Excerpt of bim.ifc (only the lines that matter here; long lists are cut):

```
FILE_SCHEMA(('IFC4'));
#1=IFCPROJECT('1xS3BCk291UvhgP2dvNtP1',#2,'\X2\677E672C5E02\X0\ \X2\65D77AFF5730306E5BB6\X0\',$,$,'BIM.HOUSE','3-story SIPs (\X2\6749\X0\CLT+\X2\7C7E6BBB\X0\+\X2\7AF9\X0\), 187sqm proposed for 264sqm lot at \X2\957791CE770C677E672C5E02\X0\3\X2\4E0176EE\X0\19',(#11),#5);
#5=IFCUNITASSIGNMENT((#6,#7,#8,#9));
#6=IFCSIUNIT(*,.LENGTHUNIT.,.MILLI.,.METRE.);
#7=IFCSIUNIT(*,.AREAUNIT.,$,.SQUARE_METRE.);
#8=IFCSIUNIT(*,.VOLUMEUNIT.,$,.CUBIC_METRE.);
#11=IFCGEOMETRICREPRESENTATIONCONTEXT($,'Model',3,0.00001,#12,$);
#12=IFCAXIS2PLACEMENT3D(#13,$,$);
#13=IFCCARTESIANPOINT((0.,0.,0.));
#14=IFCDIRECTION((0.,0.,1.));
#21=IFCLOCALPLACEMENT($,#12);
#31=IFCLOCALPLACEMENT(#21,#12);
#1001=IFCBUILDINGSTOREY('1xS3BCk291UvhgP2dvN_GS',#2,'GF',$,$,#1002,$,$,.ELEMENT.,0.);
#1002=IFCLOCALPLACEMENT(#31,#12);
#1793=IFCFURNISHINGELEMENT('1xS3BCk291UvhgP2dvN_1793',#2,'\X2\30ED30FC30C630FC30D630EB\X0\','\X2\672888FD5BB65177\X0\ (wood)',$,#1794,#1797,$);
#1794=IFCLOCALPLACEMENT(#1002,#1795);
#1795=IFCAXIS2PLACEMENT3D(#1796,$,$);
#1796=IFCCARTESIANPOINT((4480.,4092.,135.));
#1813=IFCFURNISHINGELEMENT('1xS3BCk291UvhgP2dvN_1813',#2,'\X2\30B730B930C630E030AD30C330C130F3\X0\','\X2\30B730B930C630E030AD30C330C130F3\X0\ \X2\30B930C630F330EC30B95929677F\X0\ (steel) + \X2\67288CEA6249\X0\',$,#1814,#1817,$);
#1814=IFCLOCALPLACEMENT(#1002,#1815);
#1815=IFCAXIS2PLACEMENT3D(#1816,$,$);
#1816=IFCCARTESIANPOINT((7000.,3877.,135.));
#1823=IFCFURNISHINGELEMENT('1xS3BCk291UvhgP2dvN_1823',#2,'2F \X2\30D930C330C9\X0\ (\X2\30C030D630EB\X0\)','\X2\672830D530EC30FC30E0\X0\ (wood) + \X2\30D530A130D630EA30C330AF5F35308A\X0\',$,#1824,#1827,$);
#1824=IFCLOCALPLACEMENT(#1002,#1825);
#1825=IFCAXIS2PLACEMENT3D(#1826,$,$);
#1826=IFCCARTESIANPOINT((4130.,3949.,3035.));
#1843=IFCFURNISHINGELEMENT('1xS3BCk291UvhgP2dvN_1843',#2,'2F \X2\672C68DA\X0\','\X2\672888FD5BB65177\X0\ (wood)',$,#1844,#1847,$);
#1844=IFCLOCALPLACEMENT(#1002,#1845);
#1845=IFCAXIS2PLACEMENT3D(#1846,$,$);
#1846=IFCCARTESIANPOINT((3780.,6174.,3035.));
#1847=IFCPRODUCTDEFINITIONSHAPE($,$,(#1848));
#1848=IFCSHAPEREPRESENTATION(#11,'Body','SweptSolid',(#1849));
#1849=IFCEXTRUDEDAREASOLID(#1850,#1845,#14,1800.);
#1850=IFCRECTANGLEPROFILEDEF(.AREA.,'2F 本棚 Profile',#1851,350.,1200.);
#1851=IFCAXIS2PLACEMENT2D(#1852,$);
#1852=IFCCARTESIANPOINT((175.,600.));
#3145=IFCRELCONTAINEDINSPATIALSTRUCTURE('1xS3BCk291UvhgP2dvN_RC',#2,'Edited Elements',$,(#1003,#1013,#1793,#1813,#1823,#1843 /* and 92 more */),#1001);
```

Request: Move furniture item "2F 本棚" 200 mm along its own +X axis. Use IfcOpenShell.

```python
import ifcopenshell
import ifcopenshell.api.geometry
import ifcopenshell.util.placement

model = ifcopenshell.open("bim.ifc")

item = model.by_guid("1xS3BCk291UvhgP2dvN_1843")
matrix = ifcopenshell.util.placement.get_local_placement(item.ObjectPlacement)
matrix[:3, 3] += matrix[:3, 0] * 200.0
ifcopenshell.api.geometry.edit_object_placement(model, product=item, matrix=matrix, is_si=False)

print(ifcopenshell.util.placement.get_local_placement(item.ObjectPlacement).round(3) + 0.0)

model.write("bim_rev.ifc")
```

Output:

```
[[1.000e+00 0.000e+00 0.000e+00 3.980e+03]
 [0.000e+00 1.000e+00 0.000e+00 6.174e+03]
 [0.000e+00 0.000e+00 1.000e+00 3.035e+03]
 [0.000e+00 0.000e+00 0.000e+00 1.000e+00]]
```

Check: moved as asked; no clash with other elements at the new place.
